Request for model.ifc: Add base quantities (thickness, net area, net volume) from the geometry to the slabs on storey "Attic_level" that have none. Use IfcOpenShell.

First a look at what the model holds.

```python
import ifcopenshell
import ifcopenshell.util.element
import ifcopenshell.util.unit

model = ifcopenshell.open("model.ifc")
print(model.schema)
for unit_type in ("LENGTHUNIT", "AREAUNIT", "VOLUMEUNIT"):
    print(unit_type, ifcopenshell.util.unit.calculate_unit_scale(model, unit_type))
storey = next(s for s in model.by_type("IfcBuildingStorey") if s.Name == "Attic_level")
slabs = [e for e in ifcopenshell.util.element.get_decomposition(storey) if e.is_a("IfcSlab")]
for e in sorted(slabs, key=lambda e: e.id()):
    print(e.id(), e.is_a(), e.Name, list(ifcopenshell.util.element.get_psets(e, qtos_only=True)), sep=" | ")
```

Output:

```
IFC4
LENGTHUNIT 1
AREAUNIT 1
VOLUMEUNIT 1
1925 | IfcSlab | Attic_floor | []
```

```python
import ifcopenshell
import ifcopenshell.api.pset
import ifcopenshell.geom
import ifcopenshell.util.element
import ifcopenshell.util.shape
import ifcopenshell.util.unit

model = ifcopenshell.open("model.ifc")
unit_scale = ifcopenshell.util.unit.calculate_unit_scale(model)
area_scale = ifcopenshell.util.unit.calculate_unit_scale(model, "AREAUNIT")
volume_scale = ifcopenshell.util.unit.calculate_unit_scale(model, "VOLUMEUNIT")
settings = ifcopenshell.geom.settings()

storey = next(s for s in model.by_type("IfcBuildingStorey") if s.Name == "Attic_level")
slabs = [e for e in ifcopenshell.util.element.get_decomposition(storey) if e.is_a("IfcSlab")]

for e in sorted(slabs, key=lambda e: e.id()):
    if ifcopenshell.util.element.get_psets(e, qtos_only=True, should_inherit=False):
        continue
    # Geometry comes back in metres, in the element's own axes.
    shape = ifcopenshell.geom.create_shape(settings, e)
    values = {
        "Width": ifcopenshell.util.shape.get_z(shape.geometry) / unit_scale,
        "NetArea": ifcopenshell.util.shape.get_footprint_area(shape.geometry) / area_scale,
        "NetVolume": ifcopenshell.util.shape.get_volume(shape.geometry) / volume_scale,
    }
    qto = ifcopenshell.api.pset.add_qto(model, product=e, name="Qto_SlabBaseQuantities")
    ifcopenshell.api.pset.edit_qto(model, qto=qto, properties=values)
    print(e.id(), {k: round(v, 3) for k, v in values.items()})

model.write("model_edited.ifc")
```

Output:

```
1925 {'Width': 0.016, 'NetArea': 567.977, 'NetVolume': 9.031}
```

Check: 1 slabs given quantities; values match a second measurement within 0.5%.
